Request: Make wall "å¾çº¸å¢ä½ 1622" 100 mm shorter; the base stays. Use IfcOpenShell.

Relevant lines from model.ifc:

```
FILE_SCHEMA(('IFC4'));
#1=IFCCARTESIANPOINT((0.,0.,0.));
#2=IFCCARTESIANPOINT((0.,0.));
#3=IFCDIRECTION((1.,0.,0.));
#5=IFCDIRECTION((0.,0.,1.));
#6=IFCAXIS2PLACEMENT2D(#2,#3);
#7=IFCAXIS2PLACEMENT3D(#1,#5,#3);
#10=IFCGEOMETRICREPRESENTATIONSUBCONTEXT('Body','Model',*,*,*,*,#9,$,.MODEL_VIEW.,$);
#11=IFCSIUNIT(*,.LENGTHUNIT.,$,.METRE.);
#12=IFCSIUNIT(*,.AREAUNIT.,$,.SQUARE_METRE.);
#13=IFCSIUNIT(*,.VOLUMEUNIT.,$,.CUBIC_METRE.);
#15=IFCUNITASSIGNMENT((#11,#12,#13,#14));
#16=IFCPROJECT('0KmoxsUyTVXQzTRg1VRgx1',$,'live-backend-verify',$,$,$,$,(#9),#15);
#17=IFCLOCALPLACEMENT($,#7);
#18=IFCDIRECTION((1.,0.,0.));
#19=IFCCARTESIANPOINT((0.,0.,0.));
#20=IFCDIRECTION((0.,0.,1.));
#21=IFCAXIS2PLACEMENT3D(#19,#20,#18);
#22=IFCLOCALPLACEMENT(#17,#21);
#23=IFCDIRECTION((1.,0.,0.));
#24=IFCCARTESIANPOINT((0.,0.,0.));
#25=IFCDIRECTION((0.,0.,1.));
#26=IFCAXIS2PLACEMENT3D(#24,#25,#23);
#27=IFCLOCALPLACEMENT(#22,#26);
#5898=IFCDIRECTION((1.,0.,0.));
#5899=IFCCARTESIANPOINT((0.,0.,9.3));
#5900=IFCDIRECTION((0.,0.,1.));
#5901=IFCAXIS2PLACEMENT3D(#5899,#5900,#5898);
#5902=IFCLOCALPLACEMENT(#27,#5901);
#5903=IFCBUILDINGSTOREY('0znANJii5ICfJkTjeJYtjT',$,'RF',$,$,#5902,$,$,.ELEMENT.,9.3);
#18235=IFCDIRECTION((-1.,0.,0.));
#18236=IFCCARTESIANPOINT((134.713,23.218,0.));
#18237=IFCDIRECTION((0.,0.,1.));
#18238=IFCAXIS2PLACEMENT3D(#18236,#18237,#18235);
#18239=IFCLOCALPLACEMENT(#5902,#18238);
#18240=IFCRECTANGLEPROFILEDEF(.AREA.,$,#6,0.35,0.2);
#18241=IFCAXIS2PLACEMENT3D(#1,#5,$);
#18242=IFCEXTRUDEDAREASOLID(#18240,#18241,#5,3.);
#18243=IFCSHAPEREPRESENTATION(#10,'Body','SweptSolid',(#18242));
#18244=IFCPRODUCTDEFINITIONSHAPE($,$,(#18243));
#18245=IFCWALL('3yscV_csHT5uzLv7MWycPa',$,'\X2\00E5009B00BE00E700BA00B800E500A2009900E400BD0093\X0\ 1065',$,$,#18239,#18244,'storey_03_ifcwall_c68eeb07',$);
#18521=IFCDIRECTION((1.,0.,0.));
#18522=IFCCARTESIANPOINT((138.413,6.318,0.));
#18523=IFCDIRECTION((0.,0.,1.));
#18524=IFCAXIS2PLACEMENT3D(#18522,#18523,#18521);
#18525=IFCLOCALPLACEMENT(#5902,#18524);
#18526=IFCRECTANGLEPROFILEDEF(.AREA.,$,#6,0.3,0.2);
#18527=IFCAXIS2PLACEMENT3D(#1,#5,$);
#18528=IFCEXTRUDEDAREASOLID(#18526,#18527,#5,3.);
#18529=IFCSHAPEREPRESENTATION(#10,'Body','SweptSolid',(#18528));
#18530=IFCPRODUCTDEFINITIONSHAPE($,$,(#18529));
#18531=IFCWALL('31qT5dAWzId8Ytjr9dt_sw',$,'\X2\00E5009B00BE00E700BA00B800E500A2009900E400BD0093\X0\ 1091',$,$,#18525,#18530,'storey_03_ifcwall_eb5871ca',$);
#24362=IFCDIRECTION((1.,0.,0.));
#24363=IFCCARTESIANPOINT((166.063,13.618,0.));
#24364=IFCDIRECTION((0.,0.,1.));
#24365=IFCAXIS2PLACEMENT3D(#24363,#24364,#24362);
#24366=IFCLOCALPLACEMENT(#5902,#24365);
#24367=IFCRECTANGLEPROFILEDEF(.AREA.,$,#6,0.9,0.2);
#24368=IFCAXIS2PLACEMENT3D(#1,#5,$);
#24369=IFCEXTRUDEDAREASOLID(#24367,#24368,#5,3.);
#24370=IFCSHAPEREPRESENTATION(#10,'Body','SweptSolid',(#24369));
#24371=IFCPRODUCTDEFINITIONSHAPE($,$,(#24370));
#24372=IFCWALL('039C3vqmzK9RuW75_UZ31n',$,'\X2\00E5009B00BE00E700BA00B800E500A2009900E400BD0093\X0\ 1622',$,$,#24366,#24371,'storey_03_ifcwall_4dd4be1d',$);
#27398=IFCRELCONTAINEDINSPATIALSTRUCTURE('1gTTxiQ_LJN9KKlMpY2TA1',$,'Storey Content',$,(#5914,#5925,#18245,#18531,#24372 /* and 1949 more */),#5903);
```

```python
import ifcopenshell
import ifcopenshell.geom
import ifcopenshell.util.representation
import ifcopenshell.util.shape
import ifcopenshell.util.unit

model = ifcopenshell.open("model.ifc")
unit_scale = ifcopenshell.util.unit.calculate_unit_scale(model)
settings = ifcopenshell.geom.settings()


def volume(element):
    """Net volume in cubic metres, openings subtracted."""
    shape = ifcopenshell.geom.create_shape(settings, element)
    return ifcopenshell.util.shape.get_volume(shape.geometry)


wall = model.by_guid("039C3vqmzK9RuW75_UZ31n")
before = volume(wall)

body = ifcopenshell.util.representation.get_representation(wall, "Model", "Body")
solid = body.Items[0]
old_height = solid.Depth
solid.Depth -= 0.1 / unit_scale
after = volume(wall)

print(f"height {old_height:g} -> {solid.Depth:g}, volume {before:.3f} -> {after:.3f} m3")

model.write("model-out.ifc")
```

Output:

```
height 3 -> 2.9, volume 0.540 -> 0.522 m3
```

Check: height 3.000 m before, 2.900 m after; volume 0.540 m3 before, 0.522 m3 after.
